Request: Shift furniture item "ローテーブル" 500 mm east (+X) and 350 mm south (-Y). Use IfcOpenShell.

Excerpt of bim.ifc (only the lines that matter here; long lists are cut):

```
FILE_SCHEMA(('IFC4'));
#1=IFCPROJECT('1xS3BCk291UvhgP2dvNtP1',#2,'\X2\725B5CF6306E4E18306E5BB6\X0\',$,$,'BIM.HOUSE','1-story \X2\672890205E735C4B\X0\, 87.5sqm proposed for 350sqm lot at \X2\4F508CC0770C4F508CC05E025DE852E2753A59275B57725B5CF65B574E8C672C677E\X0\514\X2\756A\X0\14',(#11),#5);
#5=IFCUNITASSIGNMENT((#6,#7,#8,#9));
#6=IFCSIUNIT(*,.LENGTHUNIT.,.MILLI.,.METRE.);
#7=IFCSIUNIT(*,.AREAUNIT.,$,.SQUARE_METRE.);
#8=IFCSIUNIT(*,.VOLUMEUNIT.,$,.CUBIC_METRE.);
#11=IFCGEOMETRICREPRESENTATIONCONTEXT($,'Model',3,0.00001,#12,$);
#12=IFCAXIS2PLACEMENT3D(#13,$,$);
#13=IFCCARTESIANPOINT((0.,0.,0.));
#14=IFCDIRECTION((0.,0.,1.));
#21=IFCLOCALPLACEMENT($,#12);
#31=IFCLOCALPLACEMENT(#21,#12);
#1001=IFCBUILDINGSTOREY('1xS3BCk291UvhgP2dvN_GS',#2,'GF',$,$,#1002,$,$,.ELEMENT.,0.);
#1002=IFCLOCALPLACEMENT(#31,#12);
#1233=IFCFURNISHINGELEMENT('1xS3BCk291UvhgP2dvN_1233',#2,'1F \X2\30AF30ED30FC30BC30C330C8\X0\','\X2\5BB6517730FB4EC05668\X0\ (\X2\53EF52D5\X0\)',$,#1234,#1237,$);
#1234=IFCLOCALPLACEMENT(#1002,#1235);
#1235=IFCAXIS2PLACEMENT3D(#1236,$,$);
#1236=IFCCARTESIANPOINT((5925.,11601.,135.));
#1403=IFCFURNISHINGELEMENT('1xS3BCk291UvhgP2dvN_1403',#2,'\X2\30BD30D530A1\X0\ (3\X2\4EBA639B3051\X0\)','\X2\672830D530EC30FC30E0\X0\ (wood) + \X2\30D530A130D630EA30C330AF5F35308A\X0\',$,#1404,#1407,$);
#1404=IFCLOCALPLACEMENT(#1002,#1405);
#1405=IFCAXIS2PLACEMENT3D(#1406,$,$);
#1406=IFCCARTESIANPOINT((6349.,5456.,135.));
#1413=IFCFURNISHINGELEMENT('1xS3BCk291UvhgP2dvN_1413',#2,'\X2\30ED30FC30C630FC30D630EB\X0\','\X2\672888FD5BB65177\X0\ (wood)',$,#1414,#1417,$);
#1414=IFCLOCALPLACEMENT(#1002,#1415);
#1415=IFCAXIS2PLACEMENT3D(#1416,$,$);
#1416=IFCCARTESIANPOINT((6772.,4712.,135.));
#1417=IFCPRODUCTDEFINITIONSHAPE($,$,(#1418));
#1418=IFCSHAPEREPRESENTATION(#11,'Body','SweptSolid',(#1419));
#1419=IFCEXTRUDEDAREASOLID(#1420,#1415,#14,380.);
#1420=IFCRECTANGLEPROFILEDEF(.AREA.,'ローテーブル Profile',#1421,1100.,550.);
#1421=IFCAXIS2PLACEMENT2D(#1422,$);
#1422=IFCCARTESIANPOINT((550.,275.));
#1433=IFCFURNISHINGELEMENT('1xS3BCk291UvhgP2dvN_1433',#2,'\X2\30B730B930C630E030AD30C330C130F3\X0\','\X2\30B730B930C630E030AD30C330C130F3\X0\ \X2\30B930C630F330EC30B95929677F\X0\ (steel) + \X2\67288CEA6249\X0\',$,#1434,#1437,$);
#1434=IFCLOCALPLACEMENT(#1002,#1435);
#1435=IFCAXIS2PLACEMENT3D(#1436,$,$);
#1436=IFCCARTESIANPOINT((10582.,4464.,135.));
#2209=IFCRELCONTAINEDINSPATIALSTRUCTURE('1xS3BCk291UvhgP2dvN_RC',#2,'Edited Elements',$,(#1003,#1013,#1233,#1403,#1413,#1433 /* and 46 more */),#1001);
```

```python
import ifcopenshell
import ifcopenshell.api.geometry
import ifcopenshell.util.placement

model = ifcopenshell.open("bim.ifc")

item = model.by_guid("1xS3BCk291UvhgP2dvN_1413")
matrix = ifcopenshell.util.placement.get_local_placement(item.ObjectPlacement)
matrix[0, 3] += 500.0
matrix[1, 3] -= 350.0
ifcopenshell.api.geometry.edit_object_placement(model, product=item, matrix=matrix, is_si=False)

print(ifcopenshell.util.placement.get_local_placement(item.ObjectPlacement).round(3) + 0.0)

model.write("bim_rev.ifc")
```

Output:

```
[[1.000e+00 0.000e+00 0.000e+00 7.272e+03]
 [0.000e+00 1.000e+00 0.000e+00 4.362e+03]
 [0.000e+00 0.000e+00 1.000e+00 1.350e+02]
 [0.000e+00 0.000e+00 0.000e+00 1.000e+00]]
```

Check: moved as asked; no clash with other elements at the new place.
